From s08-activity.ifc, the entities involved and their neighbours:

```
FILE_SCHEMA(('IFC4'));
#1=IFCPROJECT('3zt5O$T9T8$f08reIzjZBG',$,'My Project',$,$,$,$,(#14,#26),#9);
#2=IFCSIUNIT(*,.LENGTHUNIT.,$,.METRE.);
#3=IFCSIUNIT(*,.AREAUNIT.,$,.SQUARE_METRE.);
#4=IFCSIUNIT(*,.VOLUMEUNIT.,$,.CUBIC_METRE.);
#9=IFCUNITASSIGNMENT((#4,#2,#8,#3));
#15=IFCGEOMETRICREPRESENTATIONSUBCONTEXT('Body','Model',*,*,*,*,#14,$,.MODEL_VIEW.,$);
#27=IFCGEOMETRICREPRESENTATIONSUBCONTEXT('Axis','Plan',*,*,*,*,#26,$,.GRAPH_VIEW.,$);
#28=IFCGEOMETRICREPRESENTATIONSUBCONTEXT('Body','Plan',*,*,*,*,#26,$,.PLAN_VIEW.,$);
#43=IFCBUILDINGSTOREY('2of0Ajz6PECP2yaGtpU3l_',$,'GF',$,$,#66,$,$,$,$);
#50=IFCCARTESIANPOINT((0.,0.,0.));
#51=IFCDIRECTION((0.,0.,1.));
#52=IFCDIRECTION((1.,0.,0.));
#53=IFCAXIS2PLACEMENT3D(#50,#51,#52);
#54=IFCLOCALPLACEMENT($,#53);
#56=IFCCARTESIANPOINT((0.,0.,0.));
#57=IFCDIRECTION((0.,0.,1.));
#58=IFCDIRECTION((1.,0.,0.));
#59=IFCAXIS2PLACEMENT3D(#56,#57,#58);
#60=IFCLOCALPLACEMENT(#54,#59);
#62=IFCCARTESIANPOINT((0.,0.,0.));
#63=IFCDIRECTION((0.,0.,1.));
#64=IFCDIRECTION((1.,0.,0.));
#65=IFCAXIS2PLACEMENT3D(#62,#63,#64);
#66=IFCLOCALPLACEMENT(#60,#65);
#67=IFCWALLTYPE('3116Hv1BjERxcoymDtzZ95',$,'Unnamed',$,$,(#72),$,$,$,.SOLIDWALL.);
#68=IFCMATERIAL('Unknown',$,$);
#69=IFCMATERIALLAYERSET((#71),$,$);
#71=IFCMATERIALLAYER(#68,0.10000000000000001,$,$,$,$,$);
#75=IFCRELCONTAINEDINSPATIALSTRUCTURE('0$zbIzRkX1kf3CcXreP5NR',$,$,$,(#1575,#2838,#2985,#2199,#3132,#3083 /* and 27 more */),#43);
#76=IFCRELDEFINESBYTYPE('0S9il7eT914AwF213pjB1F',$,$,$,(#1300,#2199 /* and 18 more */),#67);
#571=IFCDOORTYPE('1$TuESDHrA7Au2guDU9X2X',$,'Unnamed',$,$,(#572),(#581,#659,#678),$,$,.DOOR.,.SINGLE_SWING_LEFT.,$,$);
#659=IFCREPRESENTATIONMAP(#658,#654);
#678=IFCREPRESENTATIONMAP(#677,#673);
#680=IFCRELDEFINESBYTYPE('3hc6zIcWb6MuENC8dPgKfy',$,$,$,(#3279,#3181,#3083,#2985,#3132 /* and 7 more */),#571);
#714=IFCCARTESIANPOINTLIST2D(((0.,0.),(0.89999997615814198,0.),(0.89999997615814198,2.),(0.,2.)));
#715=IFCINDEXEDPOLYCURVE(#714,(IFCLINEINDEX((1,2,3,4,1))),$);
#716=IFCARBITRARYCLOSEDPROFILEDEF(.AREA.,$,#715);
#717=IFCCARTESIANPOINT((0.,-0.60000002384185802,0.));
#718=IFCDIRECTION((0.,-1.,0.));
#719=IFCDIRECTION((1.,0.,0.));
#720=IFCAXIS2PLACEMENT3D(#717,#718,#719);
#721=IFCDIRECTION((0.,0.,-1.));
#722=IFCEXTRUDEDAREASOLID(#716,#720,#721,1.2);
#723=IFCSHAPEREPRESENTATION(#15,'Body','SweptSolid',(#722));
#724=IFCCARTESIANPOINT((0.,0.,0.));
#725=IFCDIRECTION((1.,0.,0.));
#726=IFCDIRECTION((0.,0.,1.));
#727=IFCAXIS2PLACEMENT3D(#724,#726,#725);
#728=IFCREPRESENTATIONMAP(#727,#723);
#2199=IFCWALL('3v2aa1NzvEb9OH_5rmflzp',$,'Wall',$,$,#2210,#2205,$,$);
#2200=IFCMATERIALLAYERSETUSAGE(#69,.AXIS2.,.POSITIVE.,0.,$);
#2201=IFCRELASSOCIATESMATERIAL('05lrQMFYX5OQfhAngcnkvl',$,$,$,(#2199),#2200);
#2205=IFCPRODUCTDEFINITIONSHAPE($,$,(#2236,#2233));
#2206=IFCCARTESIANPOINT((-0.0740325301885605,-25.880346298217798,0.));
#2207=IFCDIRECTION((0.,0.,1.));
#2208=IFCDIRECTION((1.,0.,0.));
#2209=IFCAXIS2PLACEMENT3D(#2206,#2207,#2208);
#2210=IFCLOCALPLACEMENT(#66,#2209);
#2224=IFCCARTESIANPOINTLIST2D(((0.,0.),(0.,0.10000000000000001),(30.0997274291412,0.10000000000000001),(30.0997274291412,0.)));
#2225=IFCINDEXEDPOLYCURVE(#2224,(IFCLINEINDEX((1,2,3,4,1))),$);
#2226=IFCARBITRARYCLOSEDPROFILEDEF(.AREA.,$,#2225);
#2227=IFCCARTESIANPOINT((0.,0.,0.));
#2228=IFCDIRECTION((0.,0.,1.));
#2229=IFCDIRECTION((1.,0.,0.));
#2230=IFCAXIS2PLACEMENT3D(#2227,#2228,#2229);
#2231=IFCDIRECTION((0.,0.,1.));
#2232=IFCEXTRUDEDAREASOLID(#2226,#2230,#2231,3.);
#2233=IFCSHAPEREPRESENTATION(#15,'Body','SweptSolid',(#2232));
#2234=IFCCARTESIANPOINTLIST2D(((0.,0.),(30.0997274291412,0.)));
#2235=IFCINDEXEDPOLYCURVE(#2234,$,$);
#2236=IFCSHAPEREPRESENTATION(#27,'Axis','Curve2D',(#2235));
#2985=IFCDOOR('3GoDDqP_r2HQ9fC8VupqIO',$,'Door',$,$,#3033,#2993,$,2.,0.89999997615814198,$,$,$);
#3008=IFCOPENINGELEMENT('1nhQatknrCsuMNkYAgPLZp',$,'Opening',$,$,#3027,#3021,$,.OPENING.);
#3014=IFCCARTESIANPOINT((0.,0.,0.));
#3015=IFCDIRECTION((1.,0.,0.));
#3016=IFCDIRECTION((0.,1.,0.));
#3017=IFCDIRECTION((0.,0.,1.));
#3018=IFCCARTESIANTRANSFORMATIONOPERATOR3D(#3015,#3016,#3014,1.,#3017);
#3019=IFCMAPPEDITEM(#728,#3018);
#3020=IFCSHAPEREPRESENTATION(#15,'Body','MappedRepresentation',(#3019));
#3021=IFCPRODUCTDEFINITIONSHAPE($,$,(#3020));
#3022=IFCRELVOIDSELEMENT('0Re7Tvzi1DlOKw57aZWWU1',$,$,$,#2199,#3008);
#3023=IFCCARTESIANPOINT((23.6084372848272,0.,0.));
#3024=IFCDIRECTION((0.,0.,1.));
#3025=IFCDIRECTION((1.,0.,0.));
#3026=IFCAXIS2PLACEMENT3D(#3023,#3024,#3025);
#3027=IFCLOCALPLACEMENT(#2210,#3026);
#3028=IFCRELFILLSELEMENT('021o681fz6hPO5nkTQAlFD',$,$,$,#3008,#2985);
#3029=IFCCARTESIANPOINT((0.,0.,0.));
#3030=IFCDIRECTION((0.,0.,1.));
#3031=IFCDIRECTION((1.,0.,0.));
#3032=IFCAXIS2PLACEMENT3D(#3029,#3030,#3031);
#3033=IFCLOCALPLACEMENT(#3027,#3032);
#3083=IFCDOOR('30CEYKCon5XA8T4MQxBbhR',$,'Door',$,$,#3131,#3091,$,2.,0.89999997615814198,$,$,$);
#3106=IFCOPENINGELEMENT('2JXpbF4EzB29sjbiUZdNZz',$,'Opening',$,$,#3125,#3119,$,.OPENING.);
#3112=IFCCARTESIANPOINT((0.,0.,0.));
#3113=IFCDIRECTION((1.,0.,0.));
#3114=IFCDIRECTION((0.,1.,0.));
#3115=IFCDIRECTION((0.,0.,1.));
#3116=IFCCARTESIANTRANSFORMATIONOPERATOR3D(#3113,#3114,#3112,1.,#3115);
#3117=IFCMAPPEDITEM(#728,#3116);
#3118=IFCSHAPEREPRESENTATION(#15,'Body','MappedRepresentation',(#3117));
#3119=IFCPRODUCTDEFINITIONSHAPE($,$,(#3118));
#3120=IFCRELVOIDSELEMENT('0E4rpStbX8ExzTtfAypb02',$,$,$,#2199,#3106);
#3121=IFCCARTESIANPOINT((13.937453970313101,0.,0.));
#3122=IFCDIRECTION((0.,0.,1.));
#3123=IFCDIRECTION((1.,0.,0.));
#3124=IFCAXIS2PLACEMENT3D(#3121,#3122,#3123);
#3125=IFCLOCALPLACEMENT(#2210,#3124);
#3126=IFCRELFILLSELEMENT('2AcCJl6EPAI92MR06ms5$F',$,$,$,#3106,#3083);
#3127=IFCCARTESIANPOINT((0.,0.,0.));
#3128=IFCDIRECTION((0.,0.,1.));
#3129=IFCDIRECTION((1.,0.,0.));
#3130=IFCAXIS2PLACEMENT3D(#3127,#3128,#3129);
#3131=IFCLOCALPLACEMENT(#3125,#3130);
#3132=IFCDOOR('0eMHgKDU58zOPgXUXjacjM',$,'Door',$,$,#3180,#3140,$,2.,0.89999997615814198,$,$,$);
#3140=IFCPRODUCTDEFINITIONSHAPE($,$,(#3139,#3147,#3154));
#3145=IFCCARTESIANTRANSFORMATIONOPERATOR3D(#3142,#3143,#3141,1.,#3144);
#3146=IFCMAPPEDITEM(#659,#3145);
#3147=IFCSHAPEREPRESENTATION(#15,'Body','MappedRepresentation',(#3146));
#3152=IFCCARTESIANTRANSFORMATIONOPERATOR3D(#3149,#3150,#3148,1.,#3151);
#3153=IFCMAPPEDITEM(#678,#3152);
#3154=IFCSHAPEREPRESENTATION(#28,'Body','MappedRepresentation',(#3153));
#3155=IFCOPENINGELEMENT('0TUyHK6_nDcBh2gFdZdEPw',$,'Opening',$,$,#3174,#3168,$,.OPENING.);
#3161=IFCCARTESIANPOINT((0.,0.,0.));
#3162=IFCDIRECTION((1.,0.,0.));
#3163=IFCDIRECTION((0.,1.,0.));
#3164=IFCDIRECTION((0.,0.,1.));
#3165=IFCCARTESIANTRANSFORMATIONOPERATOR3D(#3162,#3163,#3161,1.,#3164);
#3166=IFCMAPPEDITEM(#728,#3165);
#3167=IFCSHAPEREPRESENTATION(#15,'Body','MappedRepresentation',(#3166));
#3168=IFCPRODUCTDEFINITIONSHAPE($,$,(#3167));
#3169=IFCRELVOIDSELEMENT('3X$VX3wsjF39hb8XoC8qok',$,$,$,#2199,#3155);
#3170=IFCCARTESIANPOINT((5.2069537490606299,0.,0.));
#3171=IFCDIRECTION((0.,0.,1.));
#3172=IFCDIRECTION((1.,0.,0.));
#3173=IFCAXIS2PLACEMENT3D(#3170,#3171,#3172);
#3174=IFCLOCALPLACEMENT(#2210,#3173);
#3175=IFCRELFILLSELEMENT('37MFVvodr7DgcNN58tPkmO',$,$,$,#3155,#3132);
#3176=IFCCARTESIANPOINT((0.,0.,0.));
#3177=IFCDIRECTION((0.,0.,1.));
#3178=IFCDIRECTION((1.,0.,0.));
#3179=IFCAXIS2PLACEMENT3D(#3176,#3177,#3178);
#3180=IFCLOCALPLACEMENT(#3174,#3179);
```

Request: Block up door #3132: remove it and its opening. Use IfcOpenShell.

```python
import ifcopenshell
import ifcopenshell.api.feature
import ifcopenshell.api.root
import ifcopenshell.geom
import ifcopenshell.util.shape

model = ifcopenshell.open("s08-activity.ifc")
settings = ifcopenshell.geom.settings()


def volume(element):
    """Net volume in cubic metres, openings subtracted."""
    shape = ifcopenshell.geom.create_shape(settings, element)
    return ifcopenshell.util.shape.get_volume(shape.geometry)


door = model.by_id(3132)
opening = door.FillsVoids[0].RelatingOpeningElement
wall = opening.VoidsElements[0].RelatingBuildingElement
before = volume(wall)

ifcopenshell.api.root.remove_product(model, product=door)
ifcopenshell.api.feature.remove_feature(model, feature=opening)

after = volume(wall)

print(f"wall volume {before:.3f} -> {after:.3f} m3")

model.write("s08-activity-out.ifc")
```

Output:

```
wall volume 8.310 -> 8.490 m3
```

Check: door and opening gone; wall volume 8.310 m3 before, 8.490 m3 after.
